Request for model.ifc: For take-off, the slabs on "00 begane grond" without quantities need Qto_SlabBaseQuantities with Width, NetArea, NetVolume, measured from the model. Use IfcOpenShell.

First a look at what the model holds.

```python
import ifcopenshell
import ifcopenshell.util.element
import ifcopenshell.util.unit

model = ifcopenshell.open("model.ifc")
print(model.schema)
for unit_type in ("LENGTHUNIT", "AREAUNIT", "VOLUMEUNIT"):
    print(unit_type, ifcopenshell.util.unit.calculate_unit_scale(model, unit_type))
storey = next(s for s in model.by_type("IfcBuildingStorey") if s.Name == "00 begane grond")
slabs = [e for e in ifcopenshell.util.element.get_decomposition(storey) if e.is_a("IfcSlab")]
for e in sorted(slabs, key=lambda e: e.id()):
    print(e.id(), e.is_a(), e.Name, list(ifcopenshell.util.element.get_psets(e, qtos_only=True)), sep=" | ")
```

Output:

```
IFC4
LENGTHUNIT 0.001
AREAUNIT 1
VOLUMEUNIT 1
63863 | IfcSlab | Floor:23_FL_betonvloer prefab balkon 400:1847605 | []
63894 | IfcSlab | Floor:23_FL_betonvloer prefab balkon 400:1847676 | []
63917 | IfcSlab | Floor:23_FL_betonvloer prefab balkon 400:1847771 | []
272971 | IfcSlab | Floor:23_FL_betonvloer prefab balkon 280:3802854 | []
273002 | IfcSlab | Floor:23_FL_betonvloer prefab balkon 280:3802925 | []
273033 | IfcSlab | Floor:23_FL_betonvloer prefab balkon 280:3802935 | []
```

```python
import ifcopenshell
import ifcopenshell.api.pset
import ifcopenshell.geom
import ifcopenshell.util.element
import ifcopenshell.util.shape
import ifcopenshell.util.unit

model = ifcopenshell.open("model.ifc")
unit_scale = ifcopenshell.util.unit.calculate_unit_scale(model)
area_scale = ifcopenshell.util.unit.calculate_unit_scale(model, "AREAUNIT")
volume_scale = ifcopenshell.util.unit.calculate_unit_scale(model, "VOLUMEUNIT")
settings = ifcopenshell.geom.settings()

storey = next(s for s in model.by_type("IfcBuildingStorey") if s.Name == "00 begane grond")
slabs = [e for e in ifcopenshell.util.element.get_decomposition(storey) if e.is_a("IfcSlab")]

for e in sorted(slabs, key=lambda e: e.id()):
    if ifcopenshell.util.element.get_psets(e, qtos_only=True, should_inherit=False):
        continue
    # Geometry comes back in metres, in the element's own axes.
    shape = ifcopenshell.geom.create_shape(settings, e)
    values = {
        "Width": ifcopenshell.util.shape.get_z(shape.geometry) / unit_scale,
        "NetArea": ifcopenshell.util.shape.get_footprint_area(shape.geometry) / area_scale,
        "NetVolume": ifcopenshell.util.shape.get_volume(shape.geometry) / volume_scale,
    }
    qto = ifcopenshell.api.pset.add_qto(model, product=e, name="Qto_SlabBaseQuantities")
    ifcopenshell.api.pset.edit_qto(model, qto=qto, properties=values)
    print(e.id(), {k: round(v, 3) for k, v in values.items()})

model.write("model_updated.ifc")
```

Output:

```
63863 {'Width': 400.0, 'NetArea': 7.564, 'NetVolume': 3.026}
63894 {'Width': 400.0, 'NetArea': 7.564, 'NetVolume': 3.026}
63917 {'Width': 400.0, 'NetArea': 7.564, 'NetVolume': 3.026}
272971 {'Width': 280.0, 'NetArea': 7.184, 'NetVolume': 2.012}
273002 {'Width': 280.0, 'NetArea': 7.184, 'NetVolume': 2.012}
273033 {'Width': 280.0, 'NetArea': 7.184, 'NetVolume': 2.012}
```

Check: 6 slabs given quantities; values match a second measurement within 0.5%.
